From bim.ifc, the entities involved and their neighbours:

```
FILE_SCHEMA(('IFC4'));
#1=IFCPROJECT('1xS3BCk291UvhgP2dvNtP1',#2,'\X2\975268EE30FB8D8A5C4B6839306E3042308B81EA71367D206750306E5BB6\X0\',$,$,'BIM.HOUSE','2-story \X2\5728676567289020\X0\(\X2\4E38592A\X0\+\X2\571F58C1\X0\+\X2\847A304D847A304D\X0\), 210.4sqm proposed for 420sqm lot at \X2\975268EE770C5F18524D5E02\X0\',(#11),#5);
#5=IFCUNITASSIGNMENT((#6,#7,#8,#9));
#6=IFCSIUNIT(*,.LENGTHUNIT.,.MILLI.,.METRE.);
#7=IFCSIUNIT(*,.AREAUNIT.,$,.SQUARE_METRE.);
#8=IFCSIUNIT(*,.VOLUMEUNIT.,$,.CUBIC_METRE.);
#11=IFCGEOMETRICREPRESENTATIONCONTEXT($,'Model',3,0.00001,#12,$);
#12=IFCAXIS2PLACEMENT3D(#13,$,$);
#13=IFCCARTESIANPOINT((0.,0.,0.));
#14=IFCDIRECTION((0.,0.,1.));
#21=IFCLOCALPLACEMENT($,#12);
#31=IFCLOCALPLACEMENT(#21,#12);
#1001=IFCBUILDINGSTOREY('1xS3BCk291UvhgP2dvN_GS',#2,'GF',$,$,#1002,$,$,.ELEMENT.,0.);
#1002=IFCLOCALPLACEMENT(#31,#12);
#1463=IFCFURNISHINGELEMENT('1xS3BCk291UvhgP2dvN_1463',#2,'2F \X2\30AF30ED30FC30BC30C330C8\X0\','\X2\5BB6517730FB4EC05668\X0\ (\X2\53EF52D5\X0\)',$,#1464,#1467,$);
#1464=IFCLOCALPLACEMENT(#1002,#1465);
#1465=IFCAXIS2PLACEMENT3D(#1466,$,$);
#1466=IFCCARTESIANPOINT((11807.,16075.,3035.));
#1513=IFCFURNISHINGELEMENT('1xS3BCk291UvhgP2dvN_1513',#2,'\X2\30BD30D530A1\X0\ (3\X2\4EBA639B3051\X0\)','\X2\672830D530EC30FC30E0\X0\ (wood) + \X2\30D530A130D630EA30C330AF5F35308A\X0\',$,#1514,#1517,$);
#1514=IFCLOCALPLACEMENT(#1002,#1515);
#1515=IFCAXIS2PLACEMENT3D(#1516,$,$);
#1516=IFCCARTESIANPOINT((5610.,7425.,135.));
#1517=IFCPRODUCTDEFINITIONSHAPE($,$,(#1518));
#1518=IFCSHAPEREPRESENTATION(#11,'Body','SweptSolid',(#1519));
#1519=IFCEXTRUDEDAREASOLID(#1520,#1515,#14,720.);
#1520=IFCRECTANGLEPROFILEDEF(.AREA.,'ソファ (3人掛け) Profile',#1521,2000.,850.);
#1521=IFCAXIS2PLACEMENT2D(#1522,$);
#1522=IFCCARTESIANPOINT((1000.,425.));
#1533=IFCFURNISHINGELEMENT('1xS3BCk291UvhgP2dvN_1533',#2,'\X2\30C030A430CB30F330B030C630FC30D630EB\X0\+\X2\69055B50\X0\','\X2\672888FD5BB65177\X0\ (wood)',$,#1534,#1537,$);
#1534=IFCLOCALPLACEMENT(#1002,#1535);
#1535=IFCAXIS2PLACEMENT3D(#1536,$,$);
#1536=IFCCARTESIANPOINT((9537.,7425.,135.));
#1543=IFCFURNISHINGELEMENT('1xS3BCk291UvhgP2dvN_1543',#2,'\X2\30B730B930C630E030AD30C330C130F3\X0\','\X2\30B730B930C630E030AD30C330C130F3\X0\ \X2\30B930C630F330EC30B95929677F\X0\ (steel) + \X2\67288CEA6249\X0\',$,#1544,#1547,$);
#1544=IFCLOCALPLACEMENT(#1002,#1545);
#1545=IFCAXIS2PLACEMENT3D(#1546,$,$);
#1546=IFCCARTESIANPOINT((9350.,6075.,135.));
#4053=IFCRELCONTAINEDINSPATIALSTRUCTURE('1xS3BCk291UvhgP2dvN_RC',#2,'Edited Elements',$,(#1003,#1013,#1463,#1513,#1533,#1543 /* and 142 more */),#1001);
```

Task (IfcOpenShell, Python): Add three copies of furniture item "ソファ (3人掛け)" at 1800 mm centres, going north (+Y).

```python
import numpy as np
import ifcopenshell
import ifcopenshell.api.geometry
import ifcopenshell.api.root
import ifcopenshell.util.element
import ifcopenshell.util.placement
import ifcopenshell.util.unit

model = ifcopenshell.open("bim.ifc")
unit_scale = ifcopenshell.util.unit.calculate_unit_scale(model)


def reuse_history(source, copy):
    """copy_class also copies each property set's owner history, people and application; keep the originals."""
    for rel in copy.IsDefinedBy:
        if rel.is_a("IfcRelDefinesByProperties") and (history := rel.RelatingPropertyDefinition.OwnerHistory):
            rel.RelatingPropertyDefinition.OwnerHistory = source.OwnerHistory
            ifcopenshell.util.element.remove_deep2(model, history)


source = model.by_id(1513)
base = ifcopenshell.util.placement.get_local_placement(source.ObjectPlacement)
step = np.array([0.0, 1.0, 0.0]) * 1.8 / unit_scale

for i in range(1, 4):
    copy = ifcopenshell.api.root.copy_class(model, product=source)
    copy.Representation = ifcopenshell.util.element.copy_deep(
        model, source.Representation, exclude=["IfcGeometricRepresentationContext", "IfcRepresentationMap"]
    )
    reuse_history(source, copy)
    matrix = base.copy()
    matrix[:3, 3] += i * step
    print("added at", matrix[:3, 3].round(3) + 0.0)
    ifcopenshell.api.geometry.edit_object_placement(model, product=copy, matrix=matrix, is_si=False)

model.write("bim-out.ifc")
```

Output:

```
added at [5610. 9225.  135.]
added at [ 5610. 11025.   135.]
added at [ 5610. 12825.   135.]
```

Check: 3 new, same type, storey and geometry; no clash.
